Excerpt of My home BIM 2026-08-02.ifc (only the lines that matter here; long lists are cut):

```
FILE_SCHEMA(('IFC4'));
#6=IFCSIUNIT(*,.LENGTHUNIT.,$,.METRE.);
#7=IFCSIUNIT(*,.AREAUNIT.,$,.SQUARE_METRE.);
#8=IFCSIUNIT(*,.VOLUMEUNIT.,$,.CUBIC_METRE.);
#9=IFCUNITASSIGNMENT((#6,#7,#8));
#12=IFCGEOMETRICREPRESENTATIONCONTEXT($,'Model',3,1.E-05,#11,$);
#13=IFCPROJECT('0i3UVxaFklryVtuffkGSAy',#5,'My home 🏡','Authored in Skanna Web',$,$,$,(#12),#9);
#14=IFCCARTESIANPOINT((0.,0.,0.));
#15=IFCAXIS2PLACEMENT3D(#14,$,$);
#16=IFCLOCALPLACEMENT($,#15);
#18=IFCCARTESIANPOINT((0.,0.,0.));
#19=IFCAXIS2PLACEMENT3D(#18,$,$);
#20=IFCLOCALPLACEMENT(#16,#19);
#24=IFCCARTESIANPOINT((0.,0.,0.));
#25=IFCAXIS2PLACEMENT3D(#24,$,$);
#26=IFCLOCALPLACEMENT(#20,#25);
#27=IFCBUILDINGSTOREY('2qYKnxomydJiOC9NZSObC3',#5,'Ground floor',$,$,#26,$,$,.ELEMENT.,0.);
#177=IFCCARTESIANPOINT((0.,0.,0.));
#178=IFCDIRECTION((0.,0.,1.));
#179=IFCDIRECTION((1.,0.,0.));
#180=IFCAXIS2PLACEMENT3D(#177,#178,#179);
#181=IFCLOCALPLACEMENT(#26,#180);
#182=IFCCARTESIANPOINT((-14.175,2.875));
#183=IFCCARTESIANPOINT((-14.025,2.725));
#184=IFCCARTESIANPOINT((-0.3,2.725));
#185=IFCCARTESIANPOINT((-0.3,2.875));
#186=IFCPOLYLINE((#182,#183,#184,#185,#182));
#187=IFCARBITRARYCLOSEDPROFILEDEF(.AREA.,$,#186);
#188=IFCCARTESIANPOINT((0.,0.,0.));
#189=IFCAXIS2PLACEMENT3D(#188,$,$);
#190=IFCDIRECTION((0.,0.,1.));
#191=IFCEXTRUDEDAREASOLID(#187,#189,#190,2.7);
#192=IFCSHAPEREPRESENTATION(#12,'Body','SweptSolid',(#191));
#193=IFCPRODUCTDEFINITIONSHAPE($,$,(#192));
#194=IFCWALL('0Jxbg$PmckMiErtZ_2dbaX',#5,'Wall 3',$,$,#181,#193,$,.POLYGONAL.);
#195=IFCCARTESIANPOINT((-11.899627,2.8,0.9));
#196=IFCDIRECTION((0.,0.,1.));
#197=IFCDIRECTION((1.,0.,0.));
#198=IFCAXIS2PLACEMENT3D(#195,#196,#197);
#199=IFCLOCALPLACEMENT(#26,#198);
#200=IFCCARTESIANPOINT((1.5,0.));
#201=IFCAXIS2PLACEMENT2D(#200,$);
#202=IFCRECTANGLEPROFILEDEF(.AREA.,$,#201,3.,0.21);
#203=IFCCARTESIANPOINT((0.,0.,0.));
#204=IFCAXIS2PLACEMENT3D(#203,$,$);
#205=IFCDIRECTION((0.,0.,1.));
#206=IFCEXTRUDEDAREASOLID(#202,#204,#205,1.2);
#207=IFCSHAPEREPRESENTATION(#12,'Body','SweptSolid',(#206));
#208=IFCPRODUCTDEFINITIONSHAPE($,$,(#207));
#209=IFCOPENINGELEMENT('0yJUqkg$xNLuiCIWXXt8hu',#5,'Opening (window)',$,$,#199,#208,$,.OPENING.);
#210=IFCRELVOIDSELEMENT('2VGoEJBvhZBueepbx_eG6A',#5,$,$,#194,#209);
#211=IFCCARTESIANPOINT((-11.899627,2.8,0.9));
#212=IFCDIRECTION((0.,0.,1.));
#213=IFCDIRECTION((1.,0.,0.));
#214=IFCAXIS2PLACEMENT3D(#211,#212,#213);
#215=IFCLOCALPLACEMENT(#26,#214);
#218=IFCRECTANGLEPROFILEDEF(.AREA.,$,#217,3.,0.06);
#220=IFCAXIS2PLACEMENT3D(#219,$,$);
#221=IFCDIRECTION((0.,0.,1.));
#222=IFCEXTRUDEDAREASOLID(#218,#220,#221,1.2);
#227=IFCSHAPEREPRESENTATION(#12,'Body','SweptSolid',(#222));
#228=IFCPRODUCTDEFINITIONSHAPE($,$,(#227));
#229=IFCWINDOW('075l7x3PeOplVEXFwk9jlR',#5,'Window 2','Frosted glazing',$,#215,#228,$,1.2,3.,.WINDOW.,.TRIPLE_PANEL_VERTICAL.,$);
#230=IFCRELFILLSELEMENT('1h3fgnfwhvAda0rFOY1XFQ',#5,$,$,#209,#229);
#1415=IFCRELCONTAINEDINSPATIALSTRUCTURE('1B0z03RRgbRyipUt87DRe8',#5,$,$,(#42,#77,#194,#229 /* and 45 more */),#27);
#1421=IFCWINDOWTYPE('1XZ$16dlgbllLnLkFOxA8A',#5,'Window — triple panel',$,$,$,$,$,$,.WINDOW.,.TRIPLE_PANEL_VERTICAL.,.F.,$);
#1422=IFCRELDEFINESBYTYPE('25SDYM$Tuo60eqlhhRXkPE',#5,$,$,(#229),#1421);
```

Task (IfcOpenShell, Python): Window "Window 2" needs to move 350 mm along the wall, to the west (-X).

```python
import ifcopenshell
import ifcopenshell.api.geometry
import ifcopenshell.util.placement

model = ifcopenshell.open("My home BIM 2026-08-02.ifc")

window = model.by_guid("075l7x3PeOplVEXFwk9jlR")
opening = window.FillsVoids[0].RelatingOpeningElement
wall = opening.VoidsElements[0].RelatingBuildingElement

wall_matrix = ifcopenshell.util.placement.get_local_placement(wall.ObjectPlacement)
shift = wall_matrix[:3, 0] * -0.35
before = ifcopenshell.util.placement.get_local_placement(window.ObjectPlacement)[:3, 3].copy()

# The window is not placed relative to its opening, so move both.
for product in (opening, window):
    matrix = ifcopenshell.util.placement.get_local_placement(product.ObjectPlacement)
    matrix[:3, 3] += shift
    ifcopenshell.api.geometry.edit_object_placement(model, product=product, matrix=matrix, is_si=False)

after = ifcopenshell.util.placement.get_local_placement(window.ObjectPlacement)[:3, 3]
print("window moved by", (after - before).round(3) + 0.0)

model.write("My home BIM 2026-08-02-out.ifc")
```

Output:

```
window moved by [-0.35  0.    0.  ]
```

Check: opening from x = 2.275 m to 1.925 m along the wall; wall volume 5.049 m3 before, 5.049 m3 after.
